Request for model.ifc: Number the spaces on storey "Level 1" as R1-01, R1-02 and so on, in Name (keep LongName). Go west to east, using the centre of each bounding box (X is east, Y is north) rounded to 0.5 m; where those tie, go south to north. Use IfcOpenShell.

First a look at what the model holds.

```python
import ifcopenshell
import ifcopenshell.util.element
import ifcopenshell.util.placement

model = ifcopenshell.open("model.ifc")
print(model.schema)
storey = next(s for s in model.by_type("IfcBuildingStorey") if s.Name == "Level 1")
spaces = [e for e in ifcopenshell.util.element.get_decomposition(storey) if e.is_a("IfcSpace")]
for e in sorted(spaces, key=lambda e: e.id()):
    origin = ifcopenshell.util.placement.get_local_placement(e.ObjectPlacement)[:3, 3]
    print(e.id(), e.Name, e.LongName, origin.round(2) + 0.0, sep=" | ")
```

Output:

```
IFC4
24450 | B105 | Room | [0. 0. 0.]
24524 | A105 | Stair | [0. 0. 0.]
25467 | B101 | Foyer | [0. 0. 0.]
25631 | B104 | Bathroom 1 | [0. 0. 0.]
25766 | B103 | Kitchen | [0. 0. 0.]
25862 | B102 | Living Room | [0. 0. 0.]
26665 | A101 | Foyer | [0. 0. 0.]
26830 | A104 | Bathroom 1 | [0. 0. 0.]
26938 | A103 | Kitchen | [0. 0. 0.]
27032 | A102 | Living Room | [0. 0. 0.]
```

```python
import ifcopenshell
import ifcopenshell.geom
import ifcopenshell.util.element
import ifcopenshell.util.shape

model = ifcopenshell.open("model.ifc")
settings = ifcopenshell.geom.settings()
settings.set("use-world-coords", True)


def centre(element):
    shape = ifcopenshell.geom.create_shape(settings, element)
    return ifcopenshell.util.shape.get_bbox_centroid(shape.geometry)


storey = next(s for s in model.by_type("IfcBuildingStorey") if s.Name == "Level 1")
spaces = [e for e in ifcopenshell.util.element.get_decomposition(storey) if e.is_a("IfcSpace")]

# Insertion points can sit at a corner or the storey origin, so sort by the geometry (in metres).
centres = {e: centre(e) for e in spaces}
spaces.sort(key=lambda e: (round(centres[e][0] / 0.5), centres[e][1]))

for i, e in enumerate(spaces, start=1):
    number = f"R1-{i:02d}"
    e.Name = number
    print(e.id(), number)

model.write("model_updated.ifc")
```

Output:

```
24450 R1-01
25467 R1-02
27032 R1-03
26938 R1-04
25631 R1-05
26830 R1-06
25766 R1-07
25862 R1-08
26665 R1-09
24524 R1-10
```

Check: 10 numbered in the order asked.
